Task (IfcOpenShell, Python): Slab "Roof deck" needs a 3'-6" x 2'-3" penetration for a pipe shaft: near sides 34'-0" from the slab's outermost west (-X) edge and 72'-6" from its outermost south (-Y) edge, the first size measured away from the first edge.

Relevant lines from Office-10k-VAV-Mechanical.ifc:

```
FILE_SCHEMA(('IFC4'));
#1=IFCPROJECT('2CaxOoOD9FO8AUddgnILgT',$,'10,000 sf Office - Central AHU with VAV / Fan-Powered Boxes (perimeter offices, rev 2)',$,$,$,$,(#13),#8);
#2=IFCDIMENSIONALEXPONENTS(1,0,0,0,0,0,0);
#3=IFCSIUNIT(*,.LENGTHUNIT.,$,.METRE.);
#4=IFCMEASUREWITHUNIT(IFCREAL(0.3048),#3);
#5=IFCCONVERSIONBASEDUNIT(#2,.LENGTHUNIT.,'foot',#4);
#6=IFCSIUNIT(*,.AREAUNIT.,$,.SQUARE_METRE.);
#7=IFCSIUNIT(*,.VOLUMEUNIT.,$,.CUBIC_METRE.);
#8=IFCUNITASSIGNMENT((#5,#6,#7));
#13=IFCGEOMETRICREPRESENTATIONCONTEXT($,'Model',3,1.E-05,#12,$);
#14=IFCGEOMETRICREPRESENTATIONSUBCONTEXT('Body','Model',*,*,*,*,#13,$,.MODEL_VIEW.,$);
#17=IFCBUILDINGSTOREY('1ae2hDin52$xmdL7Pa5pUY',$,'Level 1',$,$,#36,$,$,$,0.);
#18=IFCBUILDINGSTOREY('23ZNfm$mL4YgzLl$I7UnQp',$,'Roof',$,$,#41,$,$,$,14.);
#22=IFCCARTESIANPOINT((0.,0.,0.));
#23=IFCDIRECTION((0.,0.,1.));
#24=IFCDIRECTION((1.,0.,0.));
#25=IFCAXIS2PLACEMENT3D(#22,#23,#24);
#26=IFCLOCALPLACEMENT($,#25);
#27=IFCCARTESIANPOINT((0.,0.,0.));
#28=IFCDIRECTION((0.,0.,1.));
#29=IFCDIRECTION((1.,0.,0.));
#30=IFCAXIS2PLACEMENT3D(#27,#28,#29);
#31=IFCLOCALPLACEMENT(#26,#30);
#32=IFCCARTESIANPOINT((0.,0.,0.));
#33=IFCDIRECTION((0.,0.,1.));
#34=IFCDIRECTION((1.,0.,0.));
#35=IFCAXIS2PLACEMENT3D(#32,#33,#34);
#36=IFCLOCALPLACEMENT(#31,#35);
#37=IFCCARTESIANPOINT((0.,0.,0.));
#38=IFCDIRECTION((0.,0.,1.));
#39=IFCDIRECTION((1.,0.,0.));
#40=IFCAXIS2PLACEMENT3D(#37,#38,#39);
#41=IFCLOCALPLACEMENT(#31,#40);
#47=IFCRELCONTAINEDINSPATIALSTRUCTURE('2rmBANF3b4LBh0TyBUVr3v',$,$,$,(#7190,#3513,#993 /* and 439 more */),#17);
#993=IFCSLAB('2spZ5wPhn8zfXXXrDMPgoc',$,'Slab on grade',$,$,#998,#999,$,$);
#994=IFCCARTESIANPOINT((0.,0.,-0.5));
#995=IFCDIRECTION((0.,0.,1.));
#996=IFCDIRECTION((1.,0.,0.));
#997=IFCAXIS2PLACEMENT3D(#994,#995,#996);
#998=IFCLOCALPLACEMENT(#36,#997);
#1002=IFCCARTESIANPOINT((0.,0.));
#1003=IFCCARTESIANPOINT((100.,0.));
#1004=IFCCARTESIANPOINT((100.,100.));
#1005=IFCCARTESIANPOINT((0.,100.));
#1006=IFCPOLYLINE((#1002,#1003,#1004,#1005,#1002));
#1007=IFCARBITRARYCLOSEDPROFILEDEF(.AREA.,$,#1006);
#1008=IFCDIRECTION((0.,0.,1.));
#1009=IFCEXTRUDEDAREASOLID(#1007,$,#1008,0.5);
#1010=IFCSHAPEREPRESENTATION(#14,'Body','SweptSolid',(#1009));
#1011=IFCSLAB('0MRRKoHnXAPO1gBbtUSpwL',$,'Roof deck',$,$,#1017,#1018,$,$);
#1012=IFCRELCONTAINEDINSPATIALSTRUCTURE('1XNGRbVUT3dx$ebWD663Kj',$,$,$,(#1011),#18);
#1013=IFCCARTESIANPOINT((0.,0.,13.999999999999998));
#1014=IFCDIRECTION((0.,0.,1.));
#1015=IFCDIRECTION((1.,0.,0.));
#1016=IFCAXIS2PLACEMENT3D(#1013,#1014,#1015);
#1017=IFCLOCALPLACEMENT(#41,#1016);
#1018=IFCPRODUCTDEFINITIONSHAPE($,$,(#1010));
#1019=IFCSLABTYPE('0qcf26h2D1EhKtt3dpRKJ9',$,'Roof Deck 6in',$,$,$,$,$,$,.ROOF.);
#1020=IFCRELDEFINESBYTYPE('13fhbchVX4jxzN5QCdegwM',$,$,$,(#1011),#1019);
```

```python
import numpy as np
import ifcopenshell
import ifcopenshell.api.feature
import ifcopenshell.api.geometry
import ifcopenshell.api.root
import ifcopenshell.geom
import ifcopenshell.util.placement
import ifcopenshell.util.representation
import ifcopenshell.util.shape
import ifcopenshell.util.unit

model = ifcopenshell.open("Office-10k-VAV-Mechanical.ifc")
unit_scale = ifcopenshell.util.unit.calculate_unit_scale(model)
settings = ifcopenshell.geom.settings()


def volume(element):
    """Net volume in cubic metres, openings subtracted."""
    shape = ifcopenshell.geom.create_shape(settings, element)
    return ifcopenshell.util.shape.get_volume(shape.geometry)


slab = model.by_id(1011)
before = volume(slab)

# Extent in the slab's own axes, in metres. The edges named are its -X and -Y sides.
slab_shape = ifcopenshell.geom.create_shape(settings, slab)
vertices = ifcopenshell.util.shape.get_vertices(slab_shape.geometry)
x_min, y_min, bottom = vertices.min(axis=0)
top = vertices[:, 2].max()

opening = ifcopenshell.api.root.create_entity(model, ifc_class="IfcOpeningElement", name="Pipe shaft opening", predefined_type="OPENING")
context = ifcopenshell.util.representation.get_context(model, "Model", "Body", "MODEL_VIEW")
width, depth = 1.0668, 0.6858
outline = [(0.0, 0.0), (width, 0.0), (width, depth), (0.0, depth), (0.0, 0.0)]
# Overshoot both faces by 50 mm so the cut is clean.
shape = ifcopenshell.api.geometry.add_slab_representation(
    model, context=context, depth=top - bottom + 0.1, polyline=outline
)
ifcopenshell.api.geometry.assign_representation(model, product=opening, representation=shape)

matrix = ifcopenshell.util.placement.get_local_placement(slab.ObjectPlacement)
matrix[:, 3] = matrix @ np.append(np.array([x_min + 10.3632, y_min + 22.098, bottom - 0.05]) / unit_scale, 1.0)
ifcopenshell.api.geometry.edit_object_placement(model, product=opening, matrix=matrix, is_si=False)
ifcopenshell.api.feature.add_feature(model, feature=opening, element=slab)

after = volume(slab)

print(f"slab volume {before:.3f} -> {after:.3f} m3")

model.write("Office-10k-VAV-Mechanical_edited.ifc")
```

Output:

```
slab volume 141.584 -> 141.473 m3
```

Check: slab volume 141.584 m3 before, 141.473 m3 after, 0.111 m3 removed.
